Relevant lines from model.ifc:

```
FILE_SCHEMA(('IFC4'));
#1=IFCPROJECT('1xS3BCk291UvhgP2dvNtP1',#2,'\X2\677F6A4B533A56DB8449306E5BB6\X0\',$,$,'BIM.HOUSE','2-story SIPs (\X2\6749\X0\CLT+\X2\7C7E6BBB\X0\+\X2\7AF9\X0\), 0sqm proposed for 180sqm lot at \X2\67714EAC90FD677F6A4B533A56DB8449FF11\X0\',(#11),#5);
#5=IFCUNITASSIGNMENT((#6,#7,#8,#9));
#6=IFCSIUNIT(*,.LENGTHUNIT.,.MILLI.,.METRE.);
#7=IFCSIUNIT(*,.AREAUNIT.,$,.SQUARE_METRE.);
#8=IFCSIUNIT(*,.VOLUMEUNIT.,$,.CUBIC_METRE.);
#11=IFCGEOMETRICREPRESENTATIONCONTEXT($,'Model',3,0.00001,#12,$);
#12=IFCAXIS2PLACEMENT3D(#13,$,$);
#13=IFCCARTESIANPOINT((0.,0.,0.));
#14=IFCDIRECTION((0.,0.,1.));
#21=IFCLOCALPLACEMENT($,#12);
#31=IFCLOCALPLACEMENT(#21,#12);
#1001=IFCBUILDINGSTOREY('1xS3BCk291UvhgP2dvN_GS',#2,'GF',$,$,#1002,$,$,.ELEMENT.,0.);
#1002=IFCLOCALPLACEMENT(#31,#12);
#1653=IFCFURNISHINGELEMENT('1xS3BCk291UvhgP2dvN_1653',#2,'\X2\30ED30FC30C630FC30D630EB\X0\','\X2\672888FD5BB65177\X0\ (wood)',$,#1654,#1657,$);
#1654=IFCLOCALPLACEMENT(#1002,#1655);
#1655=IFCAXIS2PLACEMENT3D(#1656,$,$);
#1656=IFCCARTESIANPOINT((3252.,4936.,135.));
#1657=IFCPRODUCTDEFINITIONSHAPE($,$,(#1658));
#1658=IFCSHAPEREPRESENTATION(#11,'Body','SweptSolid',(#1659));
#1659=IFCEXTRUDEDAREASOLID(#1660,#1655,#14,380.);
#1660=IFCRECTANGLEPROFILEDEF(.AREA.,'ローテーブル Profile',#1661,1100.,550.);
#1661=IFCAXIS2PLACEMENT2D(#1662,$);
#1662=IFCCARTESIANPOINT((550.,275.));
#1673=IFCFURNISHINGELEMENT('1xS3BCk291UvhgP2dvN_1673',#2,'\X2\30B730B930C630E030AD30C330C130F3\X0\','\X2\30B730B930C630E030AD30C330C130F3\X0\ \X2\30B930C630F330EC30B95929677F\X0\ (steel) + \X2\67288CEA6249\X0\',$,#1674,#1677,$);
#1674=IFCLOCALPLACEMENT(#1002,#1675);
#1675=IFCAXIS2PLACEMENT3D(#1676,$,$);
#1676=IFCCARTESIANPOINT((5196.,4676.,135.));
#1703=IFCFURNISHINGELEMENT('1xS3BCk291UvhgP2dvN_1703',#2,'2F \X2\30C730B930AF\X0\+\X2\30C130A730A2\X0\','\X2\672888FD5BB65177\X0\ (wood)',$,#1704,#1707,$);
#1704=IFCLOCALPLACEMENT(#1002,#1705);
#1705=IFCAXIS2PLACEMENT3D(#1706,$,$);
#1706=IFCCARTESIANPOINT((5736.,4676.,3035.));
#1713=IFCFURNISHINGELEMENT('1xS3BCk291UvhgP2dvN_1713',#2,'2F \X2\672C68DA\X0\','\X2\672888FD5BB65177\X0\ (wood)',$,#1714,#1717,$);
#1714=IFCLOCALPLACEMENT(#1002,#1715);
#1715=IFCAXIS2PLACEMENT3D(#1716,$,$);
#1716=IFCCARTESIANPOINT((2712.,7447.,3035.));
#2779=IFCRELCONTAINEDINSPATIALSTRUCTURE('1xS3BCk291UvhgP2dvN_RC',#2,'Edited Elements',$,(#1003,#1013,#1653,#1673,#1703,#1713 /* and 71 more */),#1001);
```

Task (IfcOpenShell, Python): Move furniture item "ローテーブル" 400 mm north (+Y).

```python
import ifcopenshell
import ifcopenshell.api.geometry
import ifcopenshell.util.placement

model = ifcopenshell.open("model.ifc")

item = model.by_id(1653)
matrix = ifcopenshell.util.placement.get_local_placement(item.ObjectPlacement)
matrix[1, 3] += 400.0
ifcopenshell.api.geometry.edit_object_placement(model, product=item, matrix=matrix, is_si=False)

print(ifcopenshell.util.placement.get_local_placement(item.ObjectPlacement).round(3) + 0.0)

model.write("model_rev.ifc")
```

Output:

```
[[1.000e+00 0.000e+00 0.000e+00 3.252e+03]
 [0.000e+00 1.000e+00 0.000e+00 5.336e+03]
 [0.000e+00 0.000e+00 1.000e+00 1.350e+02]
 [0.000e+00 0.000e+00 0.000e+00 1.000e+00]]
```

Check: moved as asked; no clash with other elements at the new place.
